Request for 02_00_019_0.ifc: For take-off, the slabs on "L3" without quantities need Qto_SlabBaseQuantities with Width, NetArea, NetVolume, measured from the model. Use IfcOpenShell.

First a look at what the model holds.

```python
import ifcopenshell
import ifcopenshell.util.element
import ifcopenshell.util.unit

model = ifcopenshell.open("02_00_019_0.ifc")
print(model.schema)
for unit_type in ("LENGTHUNIT", "AREAUNIT", "VOLUMEUNIT"):
    print(unit_type, ifcopenshell.util.unit.calculate_unit_scale(model, unit_type))
storey = next(s for s in model.by_type("IfcBuildingStorey") if s.Name == "L3")
slabs = [e for e in ifcopenshell.util.element.get_decomposition(storey) if e.is_a("IfcSlab")]
for e in sorted(slabs, key=lambda e: e.id()):
    print(e.id(), e.is_a(), e.Name, list(ifcopenshell.util.element.get_psets(e, qtos_only=True)), sep=" | ")
```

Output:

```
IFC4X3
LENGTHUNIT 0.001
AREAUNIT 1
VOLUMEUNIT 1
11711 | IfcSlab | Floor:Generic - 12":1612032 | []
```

```python
import ifcopenshell
import ifcopenshell.api.pset
import ifcopenshell.geom
import ifcopenshell.util.element
import ifcopenshell.util.shape
import ifcopenshell.util.unit

model = ifcopenshell.open("02_00_019_0.ifc")
unit_scale = ifcopenshell.util.unit.calculate_unit_scale(model)
area_scale = ifcopenshell.util.unit.calculate_unit_scale(model, "AREAUNIT")
volume_scale = ifcopenshell.util.unit.calculate_unit_scale(model, "VOLUMEUNIT")
settings = ifcopenshell.geom.settings()

storey = next(s for s in model.by_type("IfcBuildingStorey") if s.Name == "L3")
slabs = [e for e in ifcopenshell.util.element.get_decomposition(storey) if e.is_a("IfcSlab")]

for e in sorted(slabs, key=lambda e: e.id()):
    if ifcopenshell.util.element.get_psets(e, qtos_only=True, should_inherit=False):
        continue
    # Geometry comes back in metres, in the element's own axes.
    shape = ifcopenshell.geom.create_shape(settings, e)
    values = {
        "Width": ifcopenshell.util.shape.get_z(shape.geometry) / unit_scale,
        "NetArea": ifcopenshell.util.shape.get_footprint_area(shape.geometry) / area_scale,
        "NetVolume": ifcopenshell.util.shape.get_volume(shape.geometry) / volume_scale,
    }
    qto = ifcopenshell.api.pset.add_qto(model, product=e, name="Qto_SlabBaseQuantities")
    ifcopenshell.api.pset.edit_qto(model, qto=qto, properties=values)
    print(e.id(), {k: round(v, 3) for k, v in values.items()})

model.write("02_00_019_0_updated.ifc")
```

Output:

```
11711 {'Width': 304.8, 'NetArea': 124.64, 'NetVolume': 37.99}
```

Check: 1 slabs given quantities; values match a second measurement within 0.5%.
